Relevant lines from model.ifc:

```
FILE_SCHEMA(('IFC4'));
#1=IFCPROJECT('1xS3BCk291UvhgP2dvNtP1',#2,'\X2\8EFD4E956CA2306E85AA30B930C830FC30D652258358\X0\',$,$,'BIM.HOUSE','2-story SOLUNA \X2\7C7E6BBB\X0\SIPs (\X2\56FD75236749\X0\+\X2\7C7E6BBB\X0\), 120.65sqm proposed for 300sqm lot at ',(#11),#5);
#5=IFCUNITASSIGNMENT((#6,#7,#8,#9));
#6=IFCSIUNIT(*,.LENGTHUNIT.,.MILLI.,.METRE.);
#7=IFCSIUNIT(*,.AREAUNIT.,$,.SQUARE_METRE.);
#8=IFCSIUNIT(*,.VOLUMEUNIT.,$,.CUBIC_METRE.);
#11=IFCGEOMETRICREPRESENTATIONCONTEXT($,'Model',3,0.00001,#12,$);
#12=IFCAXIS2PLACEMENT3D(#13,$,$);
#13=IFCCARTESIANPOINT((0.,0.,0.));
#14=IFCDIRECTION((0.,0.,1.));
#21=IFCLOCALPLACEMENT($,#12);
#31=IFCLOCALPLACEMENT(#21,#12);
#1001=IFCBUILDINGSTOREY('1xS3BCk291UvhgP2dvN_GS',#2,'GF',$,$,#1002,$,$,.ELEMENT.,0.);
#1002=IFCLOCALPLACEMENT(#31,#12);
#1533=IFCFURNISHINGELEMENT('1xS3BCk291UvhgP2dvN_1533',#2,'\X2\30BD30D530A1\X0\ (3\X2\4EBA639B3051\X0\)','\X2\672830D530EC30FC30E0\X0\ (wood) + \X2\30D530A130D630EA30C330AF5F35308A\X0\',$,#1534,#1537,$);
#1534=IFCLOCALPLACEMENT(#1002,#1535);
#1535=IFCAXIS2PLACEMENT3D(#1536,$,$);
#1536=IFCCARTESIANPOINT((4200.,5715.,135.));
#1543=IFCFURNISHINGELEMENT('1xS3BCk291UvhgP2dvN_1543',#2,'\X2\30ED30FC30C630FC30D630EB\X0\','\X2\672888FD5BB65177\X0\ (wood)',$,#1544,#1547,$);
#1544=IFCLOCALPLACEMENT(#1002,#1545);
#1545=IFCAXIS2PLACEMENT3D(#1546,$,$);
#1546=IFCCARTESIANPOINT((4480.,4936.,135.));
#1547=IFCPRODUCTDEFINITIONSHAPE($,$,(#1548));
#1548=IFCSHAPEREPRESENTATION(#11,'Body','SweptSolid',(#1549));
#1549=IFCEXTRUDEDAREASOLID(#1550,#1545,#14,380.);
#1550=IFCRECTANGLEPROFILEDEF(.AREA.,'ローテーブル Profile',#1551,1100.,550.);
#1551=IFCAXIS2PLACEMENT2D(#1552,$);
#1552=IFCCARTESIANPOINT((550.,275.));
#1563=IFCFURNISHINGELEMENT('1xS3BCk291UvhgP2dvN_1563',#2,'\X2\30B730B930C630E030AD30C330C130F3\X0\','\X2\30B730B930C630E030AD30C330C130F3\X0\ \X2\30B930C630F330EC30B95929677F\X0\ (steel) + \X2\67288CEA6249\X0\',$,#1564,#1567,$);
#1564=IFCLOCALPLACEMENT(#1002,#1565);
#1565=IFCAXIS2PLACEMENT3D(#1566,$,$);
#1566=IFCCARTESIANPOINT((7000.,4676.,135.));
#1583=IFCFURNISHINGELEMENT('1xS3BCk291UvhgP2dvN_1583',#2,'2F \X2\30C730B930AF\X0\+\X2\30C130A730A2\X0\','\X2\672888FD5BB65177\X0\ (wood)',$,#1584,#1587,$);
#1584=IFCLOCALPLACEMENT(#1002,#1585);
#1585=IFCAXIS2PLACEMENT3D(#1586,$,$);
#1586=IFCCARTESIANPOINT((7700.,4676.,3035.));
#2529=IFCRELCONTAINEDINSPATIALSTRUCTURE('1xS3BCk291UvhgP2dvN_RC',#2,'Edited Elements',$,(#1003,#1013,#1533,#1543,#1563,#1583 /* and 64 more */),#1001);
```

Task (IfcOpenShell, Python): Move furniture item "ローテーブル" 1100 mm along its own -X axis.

```python
import ifcopenshell
import ifcopenshell.api.geometry
import ifcopenshell.util.placement
import ifcopenshell.util.unit

model = ifcopenshell.open("model.ifc")
unit_scale = ifcopenshell.util.unit.calculate_unit_scale(model)

item = model.by_guid("1xS3BCk291UvhgP2dvN_1543")
matrix = ifcopenshell.util.placement.get_local_placement(item.ObjectPlacement)
matrix[:3, 3] -= matrix[:3, 0] * 1.1 / unit_scale
ifcopenshell.api.geometry.edit_object_placement(model, product=item, matrix=matrix, is_si=False)

print(ifcopenshell.util.placement.get_local_placement(item.ObjectPlacement).round(3) + 0.0)

model.write("model_v2.ifc")
```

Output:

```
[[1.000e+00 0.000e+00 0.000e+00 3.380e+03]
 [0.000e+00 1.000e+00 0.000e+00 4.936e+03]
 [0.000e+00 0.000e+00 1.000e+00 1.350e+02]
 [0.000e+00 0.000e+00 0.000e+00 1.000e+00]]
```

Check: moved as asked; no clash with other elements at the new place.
